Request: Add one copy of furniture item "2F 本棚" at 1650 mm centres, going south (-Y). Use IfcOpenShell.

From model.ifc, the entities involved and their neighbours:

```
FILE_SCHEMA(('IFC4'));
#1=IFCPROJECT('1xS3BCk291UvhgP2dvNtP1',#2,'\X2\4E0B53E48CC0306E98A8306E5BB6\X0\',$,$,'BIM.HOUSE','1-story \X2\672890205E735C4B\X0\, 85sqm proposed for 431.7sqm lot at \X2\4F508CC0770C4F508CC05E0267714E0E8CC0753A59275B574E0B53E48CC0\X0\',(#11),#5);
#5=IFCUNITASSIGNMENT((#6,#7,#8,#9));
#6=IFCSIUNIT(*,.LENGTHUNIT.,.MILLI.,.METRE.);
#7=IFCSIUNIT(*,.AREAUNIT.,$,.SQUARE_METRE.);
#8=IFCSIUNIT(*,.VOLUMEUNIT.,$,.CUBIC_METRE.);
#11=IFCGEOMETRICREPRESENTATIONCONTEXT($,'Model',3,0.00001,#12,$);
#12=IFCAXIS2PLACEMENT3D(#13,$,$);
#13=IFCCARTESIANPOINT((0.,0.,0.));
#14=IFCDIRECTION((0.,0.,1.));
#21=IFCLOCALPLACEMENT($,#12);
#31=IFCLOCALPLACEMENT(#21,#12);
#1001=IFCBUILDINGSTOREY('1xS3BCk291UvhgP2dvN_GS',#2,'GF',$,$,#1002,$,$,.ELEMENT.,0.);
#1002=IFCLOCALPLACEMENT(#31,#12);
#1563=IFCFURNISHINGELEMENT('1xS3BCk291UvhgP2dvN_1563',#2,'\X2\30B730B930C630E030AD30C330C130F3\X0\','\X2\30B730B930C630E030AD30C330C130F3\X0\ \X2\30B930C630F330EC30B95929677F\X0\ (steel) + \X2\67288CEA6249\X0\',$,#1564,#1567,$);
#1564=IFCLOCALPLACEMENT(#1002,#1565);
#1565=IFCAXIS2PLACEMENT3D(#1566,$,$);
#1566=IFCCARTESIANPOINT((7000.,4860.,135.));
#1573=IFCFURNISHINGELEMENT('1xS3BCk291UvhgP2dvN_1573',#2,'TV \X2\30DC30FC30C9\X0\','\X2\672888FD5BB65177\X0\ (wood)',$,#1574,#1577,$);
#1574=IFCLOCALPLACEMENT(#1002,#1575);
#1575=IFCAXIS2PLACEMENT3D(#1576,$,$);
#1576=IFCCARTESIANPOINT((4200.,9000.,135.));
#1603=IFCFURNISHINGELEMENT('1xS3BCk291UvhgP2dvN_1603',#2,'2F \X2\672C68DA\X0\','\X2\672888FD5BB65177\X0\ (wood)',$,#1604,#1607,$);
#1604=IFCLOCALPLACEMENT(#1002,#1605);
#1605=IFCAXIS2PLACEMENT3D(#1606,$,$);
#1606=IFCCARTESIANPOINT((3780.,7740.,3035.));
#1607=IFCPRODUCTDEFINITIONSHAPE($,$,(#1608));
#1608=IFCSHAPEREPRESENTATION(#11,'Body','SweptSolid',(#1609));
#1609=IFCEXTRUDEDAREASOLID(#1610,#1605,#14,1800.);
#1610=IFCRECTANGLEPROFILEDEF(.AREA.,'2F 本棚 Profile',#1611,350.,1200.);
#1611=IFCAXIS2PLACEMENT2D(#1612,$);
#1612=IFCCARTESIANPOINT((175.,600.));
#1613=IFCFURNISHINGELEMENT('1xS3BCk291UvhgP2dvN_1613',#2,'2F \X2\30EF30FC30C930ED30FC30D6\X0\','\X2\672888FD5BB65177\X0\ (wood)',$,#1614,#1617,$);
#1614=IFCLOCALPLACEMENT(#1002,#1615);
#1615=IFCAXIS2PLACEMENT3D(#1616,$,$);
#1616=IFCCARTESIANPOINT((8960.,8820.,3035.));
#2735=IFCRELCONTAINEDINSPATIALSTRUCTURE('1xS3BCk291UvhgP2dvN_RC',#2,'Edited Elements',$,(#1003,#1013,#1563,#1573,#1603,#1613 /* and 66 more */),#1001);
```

```python
import numpy as np
import ifcopenshell
import ifcopenshell.api.geometry
import ifcopenshell.api.root
import ifcopenshell.util.element
import ifcopenshell.util.placement

model = ifcopenshell.open("model.ifc")


def reuse_history(source, copy):
    """copy_class also copies each property set's owner history, people and application; keep the originals."""
    for rel in copy.IsDefinedBy:
        if rel.is_a("IfcRelDefinesByProperties") and (history := rel.RelatingPropertyDefinition.OwnerHistory):
            rel.RelatingPropertyDefinition.OwnerHistory = source.OwnerHistory
            ifcopenshell.util.element.remove_deep2(model, history)


source = model.by_guid("1xS3BCk291UvhgP2dvN_1603")
base = ifcopenshell.util.placement.get_local_placement(source.ObjectPlacement)
step = np.array([0.0, -1.0, 0.0]) * 1650.0

for i in range(1, 2):
    copy = ifcopenshell.api.root.copy_class(model, product=source)
    copy.Representation = ifcopenshell.util.element.copy_deep(
        model, source.Representation, exclude=["IfcGeometricRepresentationContext", "IfcRepresentationMap"]
    )
    reuse_history(source, copy)
    matrix = base.copy()
    matrix[:3, 3] += i * step
    print("added at", matrix[:3, 3].round(3) + 0.0)
    ifcopenshell.api.geometry.edit_object_placement(model, product=copy, matrix=matrix, is_si=False)

model.write("model_edited.ifc")
```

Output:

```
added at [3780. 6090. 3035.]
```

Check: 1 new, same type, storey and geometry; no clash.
